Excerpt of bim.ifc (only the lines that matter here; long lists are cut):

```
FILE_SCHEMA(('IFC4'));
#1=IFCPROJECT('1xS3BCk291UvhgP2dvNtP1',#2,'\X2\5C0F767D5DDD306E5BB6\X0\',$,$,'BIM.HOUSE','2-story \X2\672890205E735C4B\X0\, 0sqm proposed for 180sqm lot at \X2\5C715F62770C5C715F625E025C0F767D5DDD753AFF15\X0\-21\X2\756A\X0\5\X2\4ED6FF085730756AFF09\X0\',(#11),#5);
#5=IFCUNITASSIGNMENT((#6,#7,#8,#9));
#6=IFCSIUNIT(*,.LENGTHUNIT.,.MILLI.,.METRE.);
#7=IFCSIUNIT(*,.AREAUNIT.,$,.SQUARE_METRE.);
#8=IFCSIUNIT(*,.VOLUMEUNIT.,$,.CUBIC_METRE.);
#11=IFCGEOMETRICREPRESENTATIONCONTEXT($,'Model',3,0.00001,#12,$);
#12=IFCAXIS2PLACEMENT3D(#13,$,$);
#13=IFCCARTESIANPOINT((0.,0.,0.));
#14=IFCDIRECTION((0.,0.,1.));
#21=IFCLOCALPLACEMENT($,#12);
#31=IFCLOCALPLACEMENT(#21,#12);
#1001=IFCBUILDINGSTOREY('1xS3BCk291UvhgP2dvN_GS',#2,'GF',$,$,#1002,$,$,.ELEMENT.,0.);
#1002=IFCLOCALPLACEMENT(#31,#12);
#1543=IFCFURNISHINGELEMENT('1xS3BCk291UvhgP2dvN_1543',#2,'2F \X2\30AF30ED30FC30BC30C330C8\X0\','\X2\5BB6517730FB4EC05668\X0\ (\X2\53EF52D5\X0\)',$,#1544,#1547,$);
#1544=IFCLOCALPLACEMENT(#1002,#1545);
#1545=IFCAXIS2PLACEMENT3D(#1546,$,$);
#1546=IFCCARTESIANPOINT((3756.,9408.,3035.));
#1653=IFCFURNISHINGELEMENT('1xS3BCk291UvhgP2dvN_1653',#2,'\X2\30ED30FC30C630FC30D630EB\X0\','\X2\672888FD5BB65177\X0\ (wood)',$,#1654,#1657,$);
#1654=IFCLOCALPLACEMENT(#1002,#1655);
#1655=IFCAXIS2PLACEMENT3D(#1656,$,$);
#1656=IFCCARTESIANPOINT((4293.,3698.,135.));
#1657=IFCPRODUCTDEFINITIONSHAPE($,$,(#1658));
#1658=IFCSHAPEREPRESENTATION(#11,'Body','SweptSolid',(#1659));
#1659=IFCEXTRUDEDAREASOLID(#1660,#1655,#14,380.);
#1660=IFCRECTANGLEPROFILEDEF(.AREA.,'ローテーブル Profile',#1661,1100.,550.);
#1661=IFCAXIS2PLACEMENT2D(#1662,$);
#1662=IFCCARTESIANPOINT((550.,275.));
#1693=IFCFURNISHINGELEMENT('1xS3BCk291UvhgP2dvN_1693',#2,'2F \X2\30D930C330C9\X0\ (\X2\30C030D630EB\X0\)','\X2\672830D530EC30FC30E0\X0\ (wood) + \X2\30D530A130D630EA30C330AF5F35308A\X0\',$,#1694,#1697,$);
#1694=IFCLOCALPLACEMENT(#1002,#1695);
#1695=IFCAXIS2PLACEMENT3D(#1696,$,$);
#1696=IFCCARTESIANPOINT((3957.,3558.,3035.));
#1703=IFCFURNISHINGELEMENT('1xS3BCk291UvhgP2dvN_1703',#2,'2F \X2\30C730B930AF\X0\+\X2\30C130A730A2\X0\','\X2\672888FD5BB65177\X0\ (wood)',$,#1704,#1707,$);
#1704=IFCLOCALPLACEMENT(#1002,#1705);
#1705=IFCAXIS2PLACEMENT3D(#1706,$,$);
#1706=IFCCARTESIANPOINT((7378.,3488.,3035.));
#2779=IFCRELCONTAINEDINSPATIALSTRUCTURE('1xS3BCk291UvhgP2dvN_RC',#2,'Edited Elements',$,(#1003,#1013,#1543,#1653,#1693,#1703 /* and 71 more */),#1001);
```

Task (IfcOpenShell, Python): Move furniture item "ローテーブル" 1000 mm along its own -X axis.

```python
import ifcopenshell
import ifcopenshell.api.geometry
import ifcopenshell.util.placement
import ifcopenshell.util.unit

model = ifcopenshell.open("bim.ifc")
unit_scale = ifcopenshell.util.unit.calculate_unit_scale(model)

item = model.by_guid("1xS3BCk291UvhgP2dvN_1653")
matrix = ifcopenshell.util.placement.get_local_placement(item.ObjectPlacement)
matrix[:3, 3] -= matrix[:3, 0] * 1 / unit_scale
ifcopenshell.api.geometry.edit_object_placement(model, product=item, matrix=matrix, is_si=False)

print(ifcopenshell.util.placement.get_local_placement(item.ObjectPlacement).round(3) + 0.0)

model.write("bim_rev.ifc")
```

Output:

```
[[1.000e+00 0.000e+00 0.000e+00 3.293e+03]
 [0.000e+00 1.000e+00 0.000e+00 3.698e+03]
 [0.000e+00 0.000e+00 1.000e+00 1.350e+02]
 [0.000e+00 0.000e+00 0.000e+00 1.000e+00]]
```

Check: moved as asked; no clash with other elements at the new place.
